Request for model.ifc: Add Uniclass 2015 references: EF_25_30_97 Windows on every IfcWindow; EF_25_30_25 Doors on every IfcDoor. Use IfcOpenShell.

First a look at what the model holds.

```python
import ifcopenshell

model = ifcopenshell.open("model.ifc")
print(model.schema)
print("classifications:", [c.Name for c in model.by_type("IfcClassification")])
for ifc_class in ("IfcDoor", "IfcRoof", "IfcStair", "IfcWall", "IfcWindow"):
    print(ifc_class, len(model.by_type(ifc_class)))
```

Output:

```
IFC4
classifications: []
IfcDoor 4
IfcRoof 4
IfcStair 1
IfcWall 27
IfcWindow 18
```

```python
import ifcopenshell
import ifcopenshell.api.classification

model = ifcopenshell.open("model.ifc")

system = ifcopenshell.api.classification.add_classification(model, classification="Uniclass 2015")

codes = {
    "IfcWindow": ("EF_25_30_97", "Windows"),
    "IfcDoor": ("EF_25_30_25", "Doors"),
}
for ifc_class, (code, name) in codes.items():
    products = model.by_type(ifc_class)
    ifcopenshell.api.classification.add_reference(
        model, products=products, classification=system, identification=code, name=name
    )
    print(code, len(products))

model.write("model_updated.ifc")
```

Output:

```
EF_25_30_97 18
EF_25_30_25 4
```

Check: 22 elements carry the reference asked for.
